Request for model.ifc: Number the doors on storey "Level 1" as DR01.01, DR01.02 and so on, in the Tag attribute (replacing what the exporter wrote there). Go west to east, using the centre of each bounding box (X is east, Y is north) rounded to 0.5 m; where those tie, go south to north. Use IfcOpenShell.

First a look at what the model holds.

```python
import ifcopenshell
import ifcopenshell.util.element
import ifcopenshell.util.placement

model = ifcopenshell.open("model.ifc")
print(model.schema)
storey = next(s for s in model.by_type("IfcBuildingStorey") if s.Name == "Level 1")
doors = [e for e in ifcopenshell.util.element.get_decomposition(storey) if e.is_a("IfcDoor")]
for e in sorted(doors, key=lambda e: e.id()):
    origin = ifcopenshell.util.placement.get_local_placement(e.ObjectPlacement)[:3, 3]
    print(e.id(), e.Tag, e.Name, origin.round(2) + 0.0, sep=" | ")
```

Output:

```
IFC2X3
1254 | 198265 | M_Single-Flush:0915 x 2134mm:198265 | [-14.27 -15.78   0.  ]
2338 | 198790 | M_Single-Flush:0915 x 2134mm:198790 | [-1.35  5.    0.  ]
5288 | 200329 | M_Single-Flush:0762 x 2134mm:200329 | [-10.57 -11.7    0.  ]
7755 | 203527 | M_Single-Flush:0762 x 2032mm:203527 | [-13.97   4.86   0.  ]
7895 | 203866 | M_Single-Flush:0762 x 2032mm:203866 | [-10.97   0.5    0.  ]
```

```python
import ifcopenshell
import ifcopenshell.geom
import ifcopenshell.util.element
import ifcopenshell.util.shape

model = ifcopenshell.open("model.ifc")
settings = ifcopenshell.geom.settings()
settings.set("use-world-coords", True)


def centre(element):
    shape = ifcopenshell.geom.create_shape(settings, element)
    return ifcopenshell.util.shape.get_bbox_centroid(shape.geometry)


storey = next(s for s in model.by_type("IfcBuildingStorey") if s.Name == "Level 1")
doors = [e for e in ifcopenshell.util.element.get_decomposition(storey) if e.is_a("IfcDoor")]

# Insertion points can sit at a corner or the storey origin, so sort by the geometry (in metres).
centres = {e: centre(e) for e in doors}
doors.sort(key=lambda e: (round(centres[e][0] / 0.5), centres[e][1]))

for i, e in enumerate(doors, start=1):
    number = f"DR01.{i:02d}"
    e.Tag = number
    print(e.id(), number)

model.write("model-out.ifc")
```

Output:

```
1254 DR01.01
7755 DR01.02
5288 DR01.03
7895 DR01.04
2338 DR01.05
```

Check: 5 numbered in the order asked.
